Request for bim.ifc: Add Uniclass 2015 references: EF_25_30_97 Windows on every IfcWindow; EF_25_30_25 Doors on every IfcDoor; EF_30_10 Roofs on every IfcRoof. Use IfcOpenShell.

First a look at what the model holds.

```python
import ifcopenshell

model = ifcopenshell.open("bim.ifc")
print(model.schema)
print("classifications:", [c.Name for c in model.by_type("IfcClassification")])
for ifc_class in ("IfcDoor", "IfcRoof", "IfcStair", "IfcWall", "IfcWindow"):
    print(ifc_class, len(model.by_type(ifc_class)))
```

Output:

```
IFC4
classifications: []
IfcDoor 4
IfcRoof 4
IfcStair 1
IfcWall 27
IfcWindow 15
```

```python
import ifcopenshell
import ifcopenshell.api.classification

model = ifcopenshell.open("bim.ifc")

system = ifcopenshell.api.classification.add_classification(model, classification="Uniclass 2015")

codes = {
    "IfcWindow": ("EF_25_30_97", "Windows"),
    "IfcDoor": ("EF_25_30_25", "Doors"),
    "IfcRoof": ("EF_30_10", "Roofs"),
}
for ifc_class, (code, name) in codes.items():
    products = model.by_type(ifc_class)
    ifcopenshell.api.classification.add_reference(
        model, products=products, classification=system, identification=code, name=name
    )
    print(code, len(products))

model.write("bim-out.ifc")
```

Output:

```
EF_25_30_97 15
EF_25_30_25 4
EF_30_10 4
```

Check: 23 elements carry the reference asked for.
